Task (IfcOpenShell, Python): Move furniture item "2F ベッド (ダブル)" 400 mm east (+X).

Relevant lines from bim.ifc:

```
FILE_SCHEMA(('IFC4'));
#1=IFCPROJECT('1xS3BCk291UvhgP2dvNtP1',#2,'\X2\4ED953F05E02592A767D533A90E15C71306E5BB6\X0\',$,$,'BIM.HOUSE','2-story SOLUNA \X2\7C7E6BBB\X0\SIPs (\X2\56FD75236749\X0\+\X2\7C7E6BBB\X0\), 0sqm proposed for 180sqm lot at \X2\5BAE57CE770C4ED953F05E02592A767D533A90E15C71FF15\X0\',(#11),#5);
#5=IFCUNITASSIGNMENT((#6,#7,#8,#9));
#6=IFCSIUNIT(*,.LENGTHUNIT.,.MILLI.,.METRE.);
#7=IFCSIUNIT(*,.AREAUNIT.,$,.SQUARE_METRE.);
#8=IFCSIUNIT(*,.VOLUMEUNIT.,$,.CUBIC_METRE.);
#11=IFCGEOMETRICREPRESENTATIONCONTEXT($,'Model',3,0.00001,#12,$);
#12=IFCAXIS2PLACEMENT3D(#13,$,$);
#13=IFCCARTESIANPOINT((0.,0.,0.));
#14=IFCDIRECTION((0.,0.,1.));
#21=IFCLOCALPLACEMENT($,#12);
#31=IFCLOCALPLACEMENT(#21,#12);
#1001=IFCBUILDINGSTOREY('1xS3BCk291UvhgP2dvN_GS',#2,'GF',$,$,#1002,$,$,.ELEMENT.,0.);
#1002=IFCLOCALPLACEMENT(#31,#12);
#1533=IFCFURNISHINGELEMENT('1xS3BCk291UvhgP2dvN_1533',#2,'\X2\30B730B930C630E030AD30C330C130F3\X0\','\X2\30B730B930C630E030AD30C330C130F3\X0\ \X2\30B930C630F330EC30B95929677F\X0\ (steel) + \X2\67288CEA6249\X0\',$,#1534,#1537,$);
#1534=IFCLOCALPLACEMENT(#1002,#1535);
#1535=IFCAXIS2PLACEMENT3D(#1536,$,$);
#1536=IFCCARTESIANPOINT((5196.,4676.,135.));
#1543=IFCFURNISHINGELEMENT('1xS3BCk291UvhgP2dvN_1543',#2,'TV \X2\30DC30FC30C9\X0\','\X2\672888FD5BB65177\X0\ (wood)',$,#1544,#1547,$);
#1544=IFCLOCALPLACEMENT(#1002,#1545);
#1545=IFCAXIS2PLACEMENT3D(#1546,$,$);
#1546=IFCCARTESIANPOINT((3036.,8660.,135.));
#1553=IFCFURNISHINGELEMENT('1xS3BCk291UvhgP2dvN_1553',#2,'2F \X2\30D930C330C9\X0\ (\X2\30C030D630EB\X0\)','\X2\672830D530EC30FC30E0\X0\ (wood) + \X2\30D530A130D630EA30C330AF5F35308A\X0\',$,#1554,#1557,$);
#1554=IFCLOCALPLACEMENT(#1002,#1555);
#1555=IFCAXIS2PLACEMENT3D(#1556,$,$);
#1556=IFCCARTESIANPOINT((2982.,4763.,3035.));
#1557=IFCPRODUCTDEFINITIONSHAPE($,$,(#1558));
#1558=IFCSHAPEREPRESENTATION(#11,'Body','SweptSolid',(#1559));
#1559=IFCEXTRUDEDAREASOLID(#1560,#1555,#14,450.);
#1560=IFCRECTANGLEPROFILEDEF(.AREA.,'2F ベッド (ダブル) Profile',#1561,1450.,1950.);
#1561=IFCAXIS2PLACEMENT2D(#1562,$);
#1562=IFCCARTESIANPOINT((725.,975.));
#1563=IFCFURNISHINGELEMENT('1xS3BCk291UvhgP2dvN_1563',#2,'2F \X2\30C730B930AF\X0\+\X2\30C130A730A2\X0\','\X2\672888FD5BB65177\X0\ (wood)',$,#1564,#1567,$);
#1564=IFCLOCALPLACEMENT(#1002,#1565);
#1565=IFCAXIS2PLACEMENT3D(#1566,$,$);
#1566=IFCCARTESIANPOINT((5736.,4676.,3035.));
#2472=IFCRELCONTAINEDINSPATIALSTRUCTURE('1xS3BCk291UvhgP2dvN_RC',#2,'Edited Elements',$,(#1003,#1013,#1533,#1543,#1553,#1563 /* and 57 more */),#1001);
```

```python
import ifcopenshell
import ifcopenshell.api.geometry
import ifcopenshell.util.placement
import ifcopenshell.util.unit

model = ifcopenshell.open("bim.ifc")
unit_scale = ifcopenshell.util.unit.calculate_unit_scale(model)

item = model.by_id(1553)
matrix = ifcopenshell.util.placement.get_local_placement(item.ObjectPlacement)
matrix[0, 3] += 0.4 / unit_scale
ifcopenshell.api.geometry.edit_object_placement(model, product=item, matrix=matrix, is_si=False)

print(ifcopenshell.util.placement.get_local_placement(item.ObjectPlacement).round(3) + 0.0)

model.write("bim_edited.ifc")
```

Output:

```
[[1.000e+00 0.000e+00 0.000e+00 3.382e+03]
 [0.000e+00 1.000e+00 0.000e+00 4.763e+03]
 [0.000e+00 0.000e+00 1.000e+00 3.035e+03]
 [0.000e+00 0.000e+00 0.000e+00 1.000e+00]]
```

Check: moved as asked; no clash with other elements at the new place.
